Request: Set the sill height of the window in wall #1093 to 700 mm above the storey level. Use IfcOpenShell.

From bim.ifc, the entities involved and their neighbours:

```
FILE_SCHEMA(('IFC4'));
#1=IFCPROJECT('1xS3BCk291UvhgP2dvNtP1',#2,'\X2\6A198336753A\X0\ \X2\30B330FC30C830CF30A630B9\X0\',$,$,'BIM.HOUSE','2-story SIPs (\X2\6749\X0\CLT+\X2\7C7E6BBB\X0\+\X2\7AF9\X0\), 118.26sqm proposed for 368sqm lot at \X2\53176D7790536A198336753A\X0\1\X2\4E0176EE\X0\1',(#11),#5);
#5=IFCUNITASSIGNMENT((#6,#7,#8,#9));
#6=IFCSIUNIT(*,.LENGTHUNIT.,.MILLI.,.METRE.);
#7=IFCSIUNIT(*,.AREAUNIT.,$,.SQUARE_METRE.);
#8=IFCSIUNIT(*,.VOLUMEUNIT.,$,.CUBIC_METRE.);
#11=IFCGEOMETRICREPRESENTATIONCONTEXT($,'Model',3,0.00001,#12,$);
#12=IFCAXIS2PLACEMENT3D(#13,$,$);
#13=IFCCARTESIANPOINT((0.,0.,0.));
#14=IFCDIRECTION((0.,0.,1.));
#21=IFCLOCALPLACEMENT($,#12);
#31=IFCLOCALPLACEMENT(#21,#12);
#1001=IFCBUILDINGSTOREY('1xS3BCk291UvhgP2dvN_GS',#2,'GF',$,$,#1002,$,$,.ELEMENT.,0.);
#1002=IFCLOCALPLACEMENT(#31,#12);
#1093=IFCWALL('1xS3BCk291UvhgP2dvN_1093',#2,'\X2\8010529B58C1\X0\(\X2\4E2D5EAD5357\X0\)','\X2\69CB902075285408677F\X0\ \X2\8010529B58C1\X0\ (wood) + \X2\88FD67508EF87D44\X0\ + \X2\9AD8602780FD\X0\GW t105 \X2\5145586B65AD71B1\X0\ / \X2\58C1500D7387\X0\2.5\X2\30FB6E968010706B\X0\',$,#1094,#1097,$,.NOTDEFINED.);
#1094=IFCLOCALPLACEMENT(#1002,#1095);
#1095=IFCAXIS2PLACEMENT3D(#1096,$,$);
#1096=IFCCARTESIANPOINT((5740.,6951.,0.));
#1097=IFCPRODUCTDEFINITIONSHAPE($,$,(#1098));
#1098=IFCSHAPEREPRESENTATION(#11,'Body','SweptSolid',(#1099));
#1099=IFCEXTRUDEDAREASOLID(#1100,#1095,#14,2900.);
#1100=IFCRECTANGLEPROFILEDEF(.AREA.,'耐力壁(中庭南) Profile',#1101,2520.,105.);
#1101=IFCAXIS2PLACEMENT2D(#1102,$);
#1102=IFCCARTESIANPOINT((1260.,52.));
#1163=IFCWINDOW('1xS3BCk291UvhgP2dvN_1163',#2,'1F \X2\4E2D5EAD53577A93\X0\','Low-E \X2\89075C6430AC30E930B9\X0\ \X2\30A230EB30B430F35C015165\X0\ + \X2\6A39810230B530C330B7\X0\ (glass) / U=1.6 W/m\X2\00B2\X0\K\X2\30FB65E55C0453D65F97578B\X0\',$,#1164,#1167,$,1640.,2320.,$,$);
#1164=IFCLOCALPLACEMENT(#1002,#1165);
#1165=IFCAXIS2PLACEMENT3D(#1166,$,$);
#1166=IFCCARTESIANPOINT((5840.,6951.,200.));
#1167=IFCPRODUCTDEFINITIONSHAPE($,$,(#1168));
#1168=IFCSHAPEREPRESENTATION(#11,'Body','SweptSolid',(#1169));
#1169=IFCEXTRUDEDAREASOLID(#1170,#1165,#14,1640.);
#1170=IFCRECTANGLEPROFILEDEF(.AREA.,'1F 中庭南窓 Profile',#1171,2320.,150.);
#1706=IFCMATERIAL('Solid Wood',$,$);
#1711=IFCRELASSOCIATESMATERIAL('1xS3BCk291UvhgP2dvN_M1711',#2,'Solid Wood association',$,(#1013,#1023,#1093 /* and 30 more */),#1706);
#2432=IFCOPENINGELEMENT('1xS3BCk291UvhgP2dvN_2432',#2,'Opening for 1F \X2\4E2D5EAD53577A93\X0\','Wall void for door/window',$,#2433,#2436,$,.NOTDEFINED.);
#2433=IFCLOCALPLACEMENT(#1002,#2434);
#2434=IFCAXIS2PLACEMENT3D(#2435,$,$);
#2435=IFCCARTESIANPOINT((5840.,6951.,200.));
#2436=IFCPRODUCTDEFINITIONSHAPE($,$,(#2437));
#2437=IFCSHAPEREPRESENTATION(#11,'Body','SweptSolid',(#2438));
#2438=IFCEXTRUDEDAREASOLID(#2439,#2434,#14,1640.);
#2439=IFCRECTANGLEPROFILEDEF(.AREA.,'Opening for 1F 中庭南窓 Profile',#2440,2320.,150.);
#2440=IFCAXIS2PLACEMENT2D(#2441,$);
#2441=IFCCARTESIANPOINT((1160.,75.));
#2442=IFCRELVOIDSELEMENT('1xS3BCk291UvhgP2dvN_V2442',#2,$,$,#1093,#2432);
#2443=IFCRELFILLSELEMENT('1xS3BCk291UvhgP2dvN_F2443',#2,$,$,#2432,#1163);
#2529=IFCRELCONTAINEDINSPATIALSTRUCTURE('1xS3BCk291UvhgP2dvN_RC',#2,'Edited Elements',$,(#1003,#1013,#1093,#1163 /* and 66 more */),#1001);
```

```python
import numpy as np
import ifcopenshell
import ifcopenshell.api.geometry
import ifcopenshell.geom
import ifcopenshell.util.element
import ifcopenshell.util.placement
import ifcopenshell.util.shape
import ifcopenshell.util.unit

model = ifcopenshell.open("bim.ifc")
unit_scale = ifcopenshell.util.unit.calculate_unit_scale(model)

window = model.by_id(1163)
opening = window.FillsVoids[0].RelatingOpeningElement
storey = ifcopenshell.util.element.get_container(window, ifc_class="IfcBuildingStorey")
level = ifcopenshell.util.placement.get_local_placement(storey.ObjectPlacement)[2, 3]

# The opening's origin need not be at the sill, so measure its lowest point.
shape = ifcopenshell.geom.create_shape(ifcopenshell.geom.settings(), opening)
bottom = ifcopenshell.util.shape.get_shape_bottom_elevation(shape, shape.geometry) / unit_scale
dz = level + 0.7 / unit_scale - bottom

shift = np.array([0.0, 0.0, dz])
# The window is not placed relative to its opening, so move both.
for product in (opening, window):
    matrix = ifcopenshell.util.placement.get_local_placement(product.ObjectPlacement)
    matrix[:3, 3] += shift
    ifcopenshell.api.geometry.edit_object_placement(model, product=product, matrix=matrix, is_si=False)

print(f"moved by {dz * unit_scale:+.3f} m")

model.write("bim_rev.ifc")
```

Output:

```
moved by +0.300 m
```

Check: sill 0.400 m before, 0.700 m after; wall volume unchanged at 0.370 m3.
